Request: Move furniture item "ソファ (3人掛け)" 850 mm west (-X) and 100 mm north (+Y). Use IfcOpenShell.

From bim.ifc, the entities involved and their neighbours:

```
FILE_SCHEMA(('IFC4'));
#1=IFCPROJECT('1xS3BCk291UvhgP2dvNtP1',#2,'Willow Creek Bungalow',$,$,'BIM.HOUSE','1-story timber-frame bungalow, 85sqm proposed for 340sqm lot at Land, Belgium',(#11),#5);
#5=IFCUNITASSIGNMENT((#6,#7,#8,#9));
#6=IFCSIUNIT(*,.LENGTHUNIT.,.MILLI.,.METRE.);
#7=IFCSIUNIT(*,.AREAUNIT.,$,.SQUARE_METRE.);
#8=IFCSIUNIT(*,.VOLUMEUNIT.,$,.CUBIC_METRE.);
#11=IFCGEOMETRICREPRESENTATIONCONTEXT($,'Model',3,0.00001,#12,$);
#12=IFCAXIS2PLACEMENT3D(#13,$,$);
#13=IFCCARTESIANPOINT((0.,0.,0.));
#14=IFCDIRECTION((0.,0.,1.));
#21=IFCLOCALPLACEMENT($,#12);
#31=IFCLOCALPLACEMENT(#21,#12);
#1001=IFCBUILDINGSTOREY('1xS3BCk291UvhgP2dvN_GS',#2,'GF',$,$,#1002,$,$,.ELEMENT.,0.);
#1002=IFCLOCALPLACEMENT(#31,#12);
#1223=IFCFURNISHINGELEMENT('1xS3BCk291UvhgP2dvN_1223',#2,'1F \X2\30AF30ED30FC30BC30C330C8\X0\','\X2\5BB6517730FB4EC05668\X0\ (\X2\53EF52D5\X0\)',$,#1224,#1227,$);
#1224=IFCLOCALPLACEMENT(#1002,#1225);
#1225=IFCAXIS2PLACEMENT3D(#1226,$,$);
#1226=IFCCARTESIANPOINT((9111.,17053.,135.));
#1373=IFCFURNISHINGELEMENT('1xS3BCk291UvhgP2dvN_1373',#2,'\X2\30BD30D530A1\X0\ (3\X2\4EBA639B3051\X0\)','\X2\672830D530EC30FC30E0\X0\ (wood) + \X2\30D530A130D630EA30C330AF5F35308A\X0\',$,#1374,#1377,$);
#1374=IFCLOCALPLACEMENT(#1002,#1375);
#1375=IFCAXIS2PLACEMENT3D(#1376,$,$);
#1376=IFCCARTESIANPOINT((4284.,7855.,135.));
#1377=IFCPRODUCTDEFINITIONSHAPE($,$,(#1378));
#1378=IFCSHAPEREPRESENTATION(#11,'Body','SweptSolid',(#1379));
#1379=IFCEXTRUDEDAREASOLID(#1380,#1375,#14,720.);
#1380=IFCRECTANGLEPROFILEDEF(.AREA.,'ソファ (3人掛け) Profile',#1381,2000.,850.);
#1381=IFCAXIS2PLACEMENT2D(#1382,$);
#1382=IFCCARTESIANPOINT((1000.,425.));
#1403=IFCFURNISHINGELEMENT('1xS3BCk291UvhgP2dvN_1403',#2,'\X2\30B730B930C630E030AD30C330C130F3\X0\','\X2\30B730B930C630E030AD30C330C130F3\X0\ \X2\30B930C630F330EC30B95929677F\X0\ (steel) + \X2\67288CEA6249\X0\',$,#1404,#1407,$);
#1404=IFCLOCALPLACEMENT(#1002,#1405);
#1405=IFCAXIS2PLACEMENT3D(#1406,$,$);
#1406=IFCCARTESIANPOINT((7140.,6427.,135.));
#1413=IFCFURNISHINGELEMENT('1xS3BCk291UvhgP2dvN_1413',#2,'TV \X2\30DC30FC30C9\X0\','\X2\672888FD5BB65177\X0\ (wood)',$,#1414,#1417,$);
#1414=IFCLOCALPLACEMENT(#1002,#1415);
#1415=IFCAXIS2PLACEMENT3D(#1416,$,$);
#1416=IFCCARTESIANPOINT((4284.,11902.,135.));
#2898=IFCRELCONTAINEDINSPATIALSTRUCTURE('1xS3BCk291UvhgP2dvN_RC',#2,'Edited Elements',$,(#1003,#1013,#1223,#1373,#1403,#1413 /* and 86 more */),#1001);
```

```python
import ifcopenshell
import ifcopenshell.api.geometry
import ifcopenshell.util.placement
import ifcopenshell.util.unit

model = ifcopenshell.open("bim.ifc")
unit_scale = ifcopenshell.util.unit.calculate_unit_scale(model)

item = model.by_id(1373)
matrix = ifcopenshell.util.placement.get_local_placement(item.ObjectPlacement)
matrix[0, 3] -= 0.85 / unit_scale
matrix[1, 3] += 0.1 / unit_scale
ifcopenshell.api.geometry.edit_object_placement(model, product=item, matrix=matrix, is_si=False)

print(ifcopenshell.util.placement.get_local_placement(item.ObjectPlacement).round(3) + 0.0)

model.write("bim_v2.ifc")
```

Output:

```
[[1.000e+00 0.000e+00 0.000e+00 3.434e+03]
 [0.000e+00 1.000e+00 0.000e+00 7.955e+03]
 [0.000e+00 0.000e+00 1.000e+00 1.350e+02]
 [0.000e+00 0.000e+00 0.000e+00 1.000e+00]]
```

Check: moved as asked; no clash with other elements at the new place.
